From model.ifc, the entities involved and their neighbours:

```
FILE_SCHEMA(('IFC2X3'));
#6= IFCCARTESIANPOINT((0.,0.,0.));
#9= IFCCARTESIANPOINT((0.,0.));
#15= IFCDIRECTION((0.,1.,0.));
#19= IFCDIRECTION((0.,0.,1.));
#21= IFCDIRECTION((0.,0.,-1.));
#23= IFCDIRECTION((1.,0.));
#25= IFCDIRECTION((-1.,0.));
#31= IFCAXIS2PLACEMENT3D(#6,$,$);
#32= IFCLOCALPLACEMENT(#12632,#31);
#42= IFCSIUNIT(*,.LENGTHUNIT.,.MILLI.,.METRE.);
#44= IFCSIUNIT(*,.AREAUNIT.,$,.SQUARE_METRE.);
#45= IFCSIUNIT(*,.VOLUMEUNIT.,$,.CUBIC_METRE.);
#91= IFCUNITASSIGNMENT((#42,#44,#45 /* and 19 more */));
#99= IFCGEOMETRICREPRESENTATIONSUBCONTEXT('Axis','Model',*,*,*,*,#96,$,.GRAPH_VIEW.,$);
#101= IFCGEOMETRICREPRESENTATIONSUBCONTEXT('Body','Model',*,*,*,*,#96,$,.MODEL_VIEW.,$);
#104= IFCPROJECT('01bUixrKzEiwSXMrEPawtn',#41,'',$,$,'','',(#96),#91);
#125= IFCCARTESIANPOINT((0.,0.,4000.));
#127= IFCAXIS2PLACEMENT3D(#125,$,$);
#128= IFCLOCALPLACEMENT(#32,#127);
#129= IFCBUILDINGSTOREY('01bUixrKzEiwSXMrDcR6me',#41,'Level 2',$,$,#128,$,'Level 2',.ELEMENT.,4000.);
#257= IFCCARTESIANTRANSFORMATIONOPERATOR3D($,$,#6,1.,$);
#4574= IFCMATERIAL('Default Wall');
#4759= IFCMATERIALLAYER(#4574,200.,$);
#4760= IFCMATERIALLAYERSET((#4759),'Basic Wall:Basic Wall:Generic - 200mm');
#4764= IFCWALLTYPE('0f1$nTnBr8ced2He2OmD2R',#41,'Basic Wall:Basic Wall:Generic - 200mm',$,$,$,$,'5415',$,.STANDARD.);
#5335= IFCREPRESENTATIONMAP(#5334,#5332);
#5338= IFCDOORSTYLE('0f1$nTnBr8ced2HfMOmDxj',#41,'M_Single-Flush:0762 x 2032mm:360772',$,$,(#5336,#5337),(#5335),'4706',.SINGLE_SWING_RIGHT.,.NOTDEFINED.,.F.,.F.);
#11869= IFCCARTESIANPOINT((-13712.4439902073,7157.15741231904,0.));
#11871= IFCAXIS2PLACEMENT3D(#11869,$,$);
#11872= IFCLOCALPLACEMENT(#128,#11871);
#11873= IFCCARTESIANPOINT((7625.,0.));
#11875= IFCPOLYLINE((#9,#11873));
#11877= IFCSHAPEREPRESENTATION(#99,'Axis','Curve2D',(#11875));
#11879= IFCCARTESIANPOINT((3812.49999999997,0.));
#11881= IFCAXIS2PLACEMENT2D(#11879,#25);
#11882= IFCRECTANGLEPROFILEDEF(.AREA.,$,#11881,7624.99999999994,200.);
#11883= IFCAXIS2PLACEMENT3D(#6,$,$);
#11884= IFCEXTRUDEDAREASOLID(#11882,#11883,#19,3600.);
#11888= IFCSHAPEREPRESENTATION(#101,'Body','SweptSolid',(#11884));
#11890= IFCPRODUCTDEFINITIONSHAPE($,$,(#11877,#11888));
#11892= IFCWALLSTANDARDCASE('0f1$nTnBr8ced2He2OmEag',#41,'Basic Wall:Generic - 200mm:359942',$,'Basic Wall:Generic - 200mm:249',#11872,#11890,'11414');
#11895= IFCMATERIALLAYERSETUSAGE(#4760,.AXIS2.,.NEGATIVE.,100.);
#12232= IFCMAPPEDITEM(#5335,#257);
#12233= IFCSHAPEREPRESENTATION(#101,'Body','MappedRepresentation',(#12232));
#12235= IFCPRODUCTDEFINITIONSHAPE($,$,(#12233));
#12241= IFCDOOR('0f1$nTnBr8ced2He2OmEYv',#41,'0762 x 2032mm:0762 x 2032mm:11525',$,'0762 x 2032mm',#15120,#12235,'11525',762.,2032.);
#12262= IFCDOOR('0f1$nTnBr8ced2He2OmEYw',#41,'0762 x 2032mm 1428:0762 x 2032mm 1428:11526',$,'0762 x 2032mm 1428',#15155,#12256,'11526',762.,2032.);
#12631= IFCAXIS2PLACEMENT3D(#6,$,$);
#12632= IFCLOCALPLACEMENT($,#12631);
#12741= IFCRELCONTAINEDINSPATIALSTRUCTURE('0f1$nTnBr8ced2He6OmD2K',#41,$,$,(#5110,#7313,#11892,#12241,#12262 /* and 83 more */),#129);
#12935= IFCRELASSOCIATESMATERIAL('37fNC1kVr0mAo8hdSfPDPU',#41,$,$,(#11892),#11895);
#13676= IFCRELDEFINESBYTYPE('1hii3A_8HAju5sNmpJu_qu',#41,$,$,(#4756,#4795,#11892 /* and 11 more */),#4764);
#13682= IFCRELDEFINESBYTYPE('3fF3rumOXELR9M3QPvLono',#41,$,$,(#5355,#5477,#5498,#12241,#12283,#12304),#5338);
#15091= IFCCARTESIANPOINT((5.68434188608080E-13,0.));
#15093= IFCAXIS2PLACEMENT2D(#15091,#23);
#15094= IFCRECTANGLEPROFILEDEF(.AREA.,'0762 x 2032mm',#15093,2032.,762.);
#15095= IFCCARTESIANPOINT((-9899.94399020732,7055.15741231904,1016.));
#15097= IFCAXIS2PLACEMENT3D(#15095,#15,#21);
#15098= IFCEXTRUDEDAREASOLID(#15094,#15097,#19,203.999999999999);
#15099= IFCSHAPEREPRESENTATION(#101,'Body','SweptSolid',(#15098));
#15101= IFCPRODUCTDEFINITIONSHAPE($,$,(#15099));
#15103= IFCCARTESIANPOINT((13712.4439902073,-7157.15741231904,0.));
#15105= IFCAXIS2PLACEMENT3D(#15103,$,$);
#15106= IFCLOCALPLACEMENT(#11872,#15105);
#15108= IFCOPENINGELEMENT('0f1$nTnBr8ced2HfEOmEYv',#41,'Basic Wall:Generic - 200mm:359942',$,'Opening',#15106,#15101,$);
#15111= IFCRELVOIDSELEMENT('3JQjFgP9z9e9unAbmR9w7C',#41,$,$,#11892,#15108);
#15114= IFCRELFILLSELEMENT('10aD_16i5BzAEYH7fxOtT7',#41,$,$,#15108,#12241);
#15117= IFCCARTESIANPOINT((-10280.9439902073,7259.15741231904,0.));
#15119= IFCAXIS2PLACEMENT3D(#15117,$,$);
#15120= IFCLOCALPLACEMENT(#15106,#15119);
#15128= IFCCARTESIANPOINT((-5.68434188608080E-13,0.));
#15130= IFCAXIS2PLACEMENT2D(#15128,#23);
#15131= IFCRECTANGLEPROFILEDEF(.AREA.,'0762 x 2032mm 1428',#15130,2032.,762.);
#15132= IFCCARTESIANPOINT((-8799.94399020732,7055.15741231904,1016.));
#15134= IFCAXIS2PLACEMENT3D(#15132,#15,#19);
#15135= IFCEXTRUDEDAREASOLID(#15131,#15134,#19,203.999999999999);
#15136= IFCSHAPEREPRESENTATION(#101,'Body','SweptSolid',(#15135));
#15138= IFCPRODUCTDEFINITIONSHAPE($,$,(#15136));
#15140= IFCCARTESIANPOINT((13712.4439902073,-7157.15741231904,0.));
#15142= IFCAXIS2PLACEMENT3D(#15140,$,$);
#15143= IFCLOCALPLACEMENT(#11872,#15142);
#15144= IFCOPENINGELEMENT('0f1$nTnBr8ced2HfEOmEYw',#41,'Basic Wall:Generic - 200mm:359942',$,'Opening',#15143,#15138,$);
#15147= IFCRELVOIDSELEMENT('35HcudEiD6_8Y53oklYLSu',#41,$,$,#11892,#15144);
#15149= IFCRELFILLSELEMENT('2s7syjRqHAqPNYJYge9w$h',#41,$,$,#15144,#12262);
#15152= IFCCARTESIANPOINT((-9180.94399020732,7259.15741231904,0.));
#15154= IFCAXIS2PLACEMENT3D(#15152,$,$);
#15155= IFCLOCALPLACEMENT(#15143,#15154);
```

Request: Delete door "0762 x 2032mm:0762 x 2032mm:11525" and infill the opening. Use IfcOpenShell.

```python
import ifcopenshell
import ifcopenshell.api.feature
import ifcopenshell.api.root
import ifcopenshell.geom
import ifcopenshell.util.shape

model = ifcopenshell.open("model.ifc")
settings = ifcopenshell.geom.settings()


def volume(element):
    """Net volume in cubic metres, openings subtracted."""
    shape = ifcopenshell.geom.create_shape(settings, element)
    return ifcopenshell.util.shape.get_volume(shape.geometry)


door = model.by_guid("0f1$nTnBr8ced2He2OmEYv")
opening = door.FillsVoids[0].RelatingOpeningElement
wall = opening.VoidsElements[0].RelatingBuildingElement
before = volume(wall)

ifcopenshell.api.root.remove_product(model, product=door)
ifcopenshell.api.feature.remove_feature(model, feature=opening)

after = volume(wall)

print(f"wall volume {before:.3f} -> {after:.3f} m3")

model.write("model_edited.ifc")
```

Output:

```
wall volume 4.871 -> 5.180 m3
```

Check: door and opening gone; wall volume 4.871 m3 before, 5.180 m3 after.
